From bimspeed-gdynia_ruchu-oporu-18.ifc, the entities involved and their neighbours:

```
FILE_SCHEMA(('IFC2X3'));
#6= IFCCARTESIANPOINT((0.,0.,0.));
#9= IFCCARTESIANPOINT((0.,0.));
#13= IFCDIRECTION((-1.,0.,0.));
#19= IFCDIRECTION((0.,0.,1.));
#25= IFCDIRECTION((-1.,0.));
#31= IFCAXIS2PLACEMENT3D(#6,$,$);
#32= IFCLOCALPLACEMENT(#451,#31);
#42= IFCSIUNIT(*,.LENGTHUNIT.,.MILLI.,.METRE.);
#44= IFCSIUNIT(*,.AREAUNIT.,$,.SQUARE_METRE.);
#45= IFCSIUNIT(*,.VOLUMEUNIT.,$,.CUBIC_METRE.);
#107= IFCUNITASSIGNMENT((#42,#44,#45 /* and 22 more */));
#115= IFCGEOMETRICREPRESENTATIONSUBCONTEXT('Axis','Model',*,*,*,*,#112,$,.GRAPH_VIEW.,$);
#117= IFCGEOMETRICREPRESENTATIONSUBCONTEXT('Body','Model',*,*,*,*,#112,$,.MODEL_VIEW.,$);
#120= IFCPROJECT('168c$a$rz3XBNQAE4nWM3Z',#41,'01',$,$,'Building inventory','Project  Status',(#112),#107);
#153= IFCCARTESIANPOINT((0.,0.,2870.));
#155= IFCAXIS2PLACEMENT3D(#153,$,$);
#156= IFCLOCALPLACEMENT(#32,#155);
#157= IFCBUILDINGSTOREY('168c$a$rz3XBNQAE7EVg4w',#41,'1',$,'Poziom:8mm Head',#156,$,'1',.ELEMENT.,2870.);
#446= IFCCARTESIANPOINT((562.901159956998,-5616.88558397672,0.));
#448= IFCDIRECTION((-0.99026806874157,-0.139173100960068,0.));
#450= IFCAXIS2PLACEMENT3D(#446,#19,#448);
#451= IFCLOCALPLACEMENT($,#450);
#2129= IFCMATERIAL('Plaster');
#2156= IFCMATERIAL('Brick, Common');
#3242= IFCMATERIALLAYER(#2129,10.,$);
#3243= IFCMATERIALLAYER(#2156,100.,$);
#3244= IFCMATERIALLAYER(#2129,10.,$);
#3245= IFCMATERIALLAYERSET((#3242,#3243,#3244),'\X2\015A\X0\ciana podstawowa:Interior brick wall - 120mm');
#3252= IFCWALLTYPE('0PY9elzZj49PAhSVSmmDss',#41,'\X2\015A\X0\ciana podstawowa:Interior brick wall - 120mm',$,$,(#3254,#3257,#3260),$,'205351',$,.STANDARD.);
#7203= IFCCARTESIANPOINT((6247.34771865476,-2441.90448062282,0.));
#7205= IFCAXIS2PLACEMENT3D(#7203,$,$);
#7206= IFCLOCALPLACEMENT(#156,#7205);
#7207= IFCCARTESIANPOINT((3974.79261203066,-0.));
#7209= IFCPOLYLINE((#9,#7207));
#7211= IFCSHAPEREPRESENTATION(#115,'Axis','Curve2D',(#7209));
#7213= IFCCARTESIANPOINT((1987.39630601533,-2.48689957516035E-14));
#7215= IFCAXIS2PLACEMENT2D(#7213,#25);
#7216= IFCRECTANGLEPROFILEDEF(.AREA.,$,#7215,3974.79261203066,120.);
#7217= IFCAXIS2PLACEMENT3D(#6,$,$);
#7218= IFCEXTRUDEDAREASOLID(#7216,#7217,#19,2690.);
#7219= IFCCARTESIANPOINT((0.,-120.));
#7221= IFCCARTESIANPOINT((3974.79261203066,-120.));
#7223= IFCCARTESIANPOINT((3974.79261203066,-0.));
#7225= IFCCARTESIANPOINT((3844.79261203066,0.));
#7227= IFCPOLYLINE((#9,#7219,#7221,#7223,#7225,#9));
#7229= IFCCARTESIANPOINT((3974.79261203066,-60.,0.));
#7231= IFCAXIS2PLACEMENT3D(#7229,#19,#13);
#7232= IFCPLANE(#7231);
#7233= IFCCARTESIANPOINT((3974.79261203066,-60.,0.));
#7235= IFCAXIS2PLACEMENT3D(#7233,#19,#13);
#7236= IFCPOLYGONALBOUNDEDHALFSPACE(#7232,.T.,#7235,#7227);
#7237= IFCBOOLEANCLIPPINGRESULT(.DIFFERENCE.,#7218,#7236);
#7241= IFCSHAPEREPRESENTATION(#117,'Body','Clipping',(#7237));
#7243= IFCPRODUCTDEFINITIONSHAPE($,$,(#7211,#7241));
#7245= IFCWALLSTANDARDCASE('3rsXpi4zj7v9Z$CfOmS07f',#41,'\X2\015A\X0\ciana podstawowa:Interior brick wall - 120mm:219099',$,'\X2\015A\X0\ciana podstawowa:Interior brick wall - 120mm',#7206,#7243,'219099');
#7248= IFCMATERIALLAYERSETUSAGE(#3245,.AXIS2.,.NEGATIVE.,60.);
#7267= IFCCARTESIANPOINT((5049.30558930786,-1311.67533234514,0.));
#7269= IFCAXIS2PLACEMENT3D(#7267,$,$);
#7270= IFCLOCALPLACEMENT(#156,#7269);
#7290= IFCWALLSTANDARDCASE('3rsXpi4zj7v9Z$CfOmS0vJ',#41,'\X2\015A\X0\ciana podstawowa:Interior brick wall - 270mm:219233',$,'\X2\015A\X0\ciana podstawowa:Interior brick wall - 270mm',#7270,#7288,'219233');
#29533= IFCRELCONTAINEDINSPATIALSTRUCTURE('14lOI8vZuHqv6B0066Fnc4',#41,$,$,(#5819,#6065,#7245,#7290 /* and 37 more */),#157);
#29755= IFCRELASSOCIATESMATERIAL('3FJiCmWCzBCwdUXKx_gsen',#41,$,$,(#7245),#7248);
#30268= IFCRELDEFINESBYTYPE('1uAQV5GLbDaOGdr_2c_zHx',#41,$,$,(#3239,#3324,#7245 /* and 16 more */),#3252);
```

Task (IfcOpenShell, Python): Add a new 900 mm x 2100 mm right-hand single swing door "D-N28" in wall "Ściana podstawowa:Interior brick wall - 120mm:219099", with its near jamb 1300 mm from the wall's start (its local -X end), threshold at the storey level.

```python
import numpy as np
import ifcopenshell
import ifcopenshell.api.feature
import ifcopenshell.api.geometry
import ifcopenshell.api.root
import ifcopenshell.api.spatial
import ifcopenshell.api.type
import ifcopenshell.geom
import ifcopenshell.util.element
import ifcopenshell.util.placement
import ifcopenshell.util.representation
import ifcopenshell.util.shape
import ifcopenshell.util.unit

model = ifcopenshell.open("bimspeed-gdynia_ruchu-oporu-18.ifc")
unit_scale = ifcopenshell.util.unit.calculate_unit_scale(model)
settings = ifcopenshell.geom.settings()


def volume(element):
    """Net volume in cubic metres, openings subtracted."""
    shape = ifcopenshell.geom.create_shape(settings, element)
    return ifcopenshell.util.shape.get_volume(shape.geometry)


wall = model.by_guid("3rsXpi4zj7v9Z$CfOmS07f")
storey = ifcopenshell.util.element.get_container(wall, ifc_class="IfcBuildingStorey")
context = ifcopenshell.util.representation.get_context(model, "Model", "Body", "MODEL_VIEW")
before = volume(wall)

width, height, from_end, sill = 0.9, 2.1, 1.3, 0.0  # metres

# The wall runs along its own X axis, and the end named is its -X end.
wall_shape = ifcopenshell.geom.create_shape(settings, wall)
x, y, z = ifcopenshell.util.shape.get_vertices(wall_shape.geometry).T
start = x.min() + from_end
face, thickness = float(y.min()), float(y.max() - y.min())
wall_matrix = ifcopenshell.util.placement.get_local_placement(wall.ObjectPlacement)
level = ifcopenshell.util.placement.get_local_placement(storey.ObjectPlacement)[2, 3]


def in_wall(x, y):
    """Placement at x, y metres in the wall's axes, at sill height."""
    matrix = wall_matrix.copy()
    matrix[:, 3] = wall_matrix @ np.array([x / unit_scale, y / unit_scale, 0.0, 1.0])
    matrix[2, 3] = level + sill / unit_scale
    return matrix


# Opening: a box that overshoots both wall faces by 50 mm.
opening = ifcopenshell.api.root.create_entity(model, ifc_class="IfcOpeningElement")
box = ifcopenshell.api.geometry.add_wall_representation(
    model, context=context, length=width, height=height, thickness=thickness + 0.1
)
ifcopenshell.api.geometry.assign_representation(model, product=opening, representation=box)
ifcopenshell.api.geometry.edit_object_placement(model, product=opening, matrix=in_wall(start, face - 0.05), is_si=False)
ifcopenshell.api.feature.add_feature(model, feature=opening, element=wall)

door = ifcopenshell.api.root.create_entity(model, ifc_class="IfcDoor", name="D-N28")
door.OverallWidth, door.OverallHeight = width / unit_scale, height / unit_scale
body = ifcopenshell.api.geometry.add_door_representation(
    model,
    context=context,
    overall_width=door.OverallWidth,
    overall_height=door.OverallHeight,
    operation_type="SINGLE_SWING_RIGHT",
    lining_properties={"LiningDepth": thickness / unit_scale, "ThresholdDepth": thickness / unit_scale},
)
ifcopenshell.api.geometry.assign_representation(model, product=door, representation=body)
ifcopenshell.api.spatial.assign_container(model, products=[door], relating_structure=storey)
fills = ifcopenshell.api.feature.add_filling(model, opening=opening, element=door)
fills.OwnerHistory = door.OwnerHistory  # required in IFC2X3

# IFC2X3 keeps the operation on the door style.
style = ifcopenshell.api.root.create_entity(model, ifc_class="IfcDoorStyle", name="D-N28")
style.OperationType, style.ConstructionType = "SINGLE_SWING_RIGHT", "NOTDEFINED"
style.ParameterTakesPrecedence = style.Sizeable = False
ifcopenshell.api.type.assign_type(model, related_objects=[door], relating_type=style)

# The lining spans the wall, so the door starts at the wall face.
ifcopenshell.api.geometry.edit_object_placement(model, product=door, matrix=in_wall(start, face), is_si=False)

after = volume(wall)

print(f"wall volume {before:.3f} -> {after:.3f} m3")

model.write("bimspeed-gdynia_ruchu-oporu-18_rev.ifc")
```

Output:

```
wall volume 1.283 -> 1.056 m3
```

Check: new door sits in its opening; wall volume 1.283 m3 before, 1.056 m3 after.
